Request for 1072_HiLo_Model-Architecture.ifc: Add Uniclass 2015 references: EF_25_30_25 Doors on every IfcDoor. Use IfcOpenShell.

First a look at what the model holds.

```python
import ifcopenshell

model = ifcopenshell.open("1072_HiLo_Model-Architecture.ifc")
print(model.schema)
print("classifications:", [c.Name for c in model.by_type("IfcClassification")])
for ifc_class in ("IfcDoor", "IfcRoof", "IfcStair", "IfcWall", "IfcWindow"):
    print(ifc_class, len(model.by_type(ifc_class)))
```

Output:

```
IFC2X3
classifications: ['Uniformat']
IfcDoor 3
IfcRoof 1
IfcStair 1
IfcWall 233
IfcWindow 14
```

```python
import ifcopenshell
import ifcopenshell.api.classification

model = ifcopenshell.open("1072_HiLo_Model-Architecture.ifc")

# IFC2X3 requires Source and Edition and has no link from the project to the system.
system = model.create_entity("IfcClassification", Source="NBS", Edition="2015", Name="Uniclass 2015")

codes = {
    "IfcDoor": ("EF_25_30_25", "Doors"),
}
for ifc_class, (code, name) in codes.items():
    products = model.by_type(ifc_class)
    ifcopenshell.api.classification.add_reference(
        model, products=products, classification=system, identification=code, name=name
    )
    print(code, len(products))

model.write("1072_HiLo_Model-Architecture-out.ifc")
```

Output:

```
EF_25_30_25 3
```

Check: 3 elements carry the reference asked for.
